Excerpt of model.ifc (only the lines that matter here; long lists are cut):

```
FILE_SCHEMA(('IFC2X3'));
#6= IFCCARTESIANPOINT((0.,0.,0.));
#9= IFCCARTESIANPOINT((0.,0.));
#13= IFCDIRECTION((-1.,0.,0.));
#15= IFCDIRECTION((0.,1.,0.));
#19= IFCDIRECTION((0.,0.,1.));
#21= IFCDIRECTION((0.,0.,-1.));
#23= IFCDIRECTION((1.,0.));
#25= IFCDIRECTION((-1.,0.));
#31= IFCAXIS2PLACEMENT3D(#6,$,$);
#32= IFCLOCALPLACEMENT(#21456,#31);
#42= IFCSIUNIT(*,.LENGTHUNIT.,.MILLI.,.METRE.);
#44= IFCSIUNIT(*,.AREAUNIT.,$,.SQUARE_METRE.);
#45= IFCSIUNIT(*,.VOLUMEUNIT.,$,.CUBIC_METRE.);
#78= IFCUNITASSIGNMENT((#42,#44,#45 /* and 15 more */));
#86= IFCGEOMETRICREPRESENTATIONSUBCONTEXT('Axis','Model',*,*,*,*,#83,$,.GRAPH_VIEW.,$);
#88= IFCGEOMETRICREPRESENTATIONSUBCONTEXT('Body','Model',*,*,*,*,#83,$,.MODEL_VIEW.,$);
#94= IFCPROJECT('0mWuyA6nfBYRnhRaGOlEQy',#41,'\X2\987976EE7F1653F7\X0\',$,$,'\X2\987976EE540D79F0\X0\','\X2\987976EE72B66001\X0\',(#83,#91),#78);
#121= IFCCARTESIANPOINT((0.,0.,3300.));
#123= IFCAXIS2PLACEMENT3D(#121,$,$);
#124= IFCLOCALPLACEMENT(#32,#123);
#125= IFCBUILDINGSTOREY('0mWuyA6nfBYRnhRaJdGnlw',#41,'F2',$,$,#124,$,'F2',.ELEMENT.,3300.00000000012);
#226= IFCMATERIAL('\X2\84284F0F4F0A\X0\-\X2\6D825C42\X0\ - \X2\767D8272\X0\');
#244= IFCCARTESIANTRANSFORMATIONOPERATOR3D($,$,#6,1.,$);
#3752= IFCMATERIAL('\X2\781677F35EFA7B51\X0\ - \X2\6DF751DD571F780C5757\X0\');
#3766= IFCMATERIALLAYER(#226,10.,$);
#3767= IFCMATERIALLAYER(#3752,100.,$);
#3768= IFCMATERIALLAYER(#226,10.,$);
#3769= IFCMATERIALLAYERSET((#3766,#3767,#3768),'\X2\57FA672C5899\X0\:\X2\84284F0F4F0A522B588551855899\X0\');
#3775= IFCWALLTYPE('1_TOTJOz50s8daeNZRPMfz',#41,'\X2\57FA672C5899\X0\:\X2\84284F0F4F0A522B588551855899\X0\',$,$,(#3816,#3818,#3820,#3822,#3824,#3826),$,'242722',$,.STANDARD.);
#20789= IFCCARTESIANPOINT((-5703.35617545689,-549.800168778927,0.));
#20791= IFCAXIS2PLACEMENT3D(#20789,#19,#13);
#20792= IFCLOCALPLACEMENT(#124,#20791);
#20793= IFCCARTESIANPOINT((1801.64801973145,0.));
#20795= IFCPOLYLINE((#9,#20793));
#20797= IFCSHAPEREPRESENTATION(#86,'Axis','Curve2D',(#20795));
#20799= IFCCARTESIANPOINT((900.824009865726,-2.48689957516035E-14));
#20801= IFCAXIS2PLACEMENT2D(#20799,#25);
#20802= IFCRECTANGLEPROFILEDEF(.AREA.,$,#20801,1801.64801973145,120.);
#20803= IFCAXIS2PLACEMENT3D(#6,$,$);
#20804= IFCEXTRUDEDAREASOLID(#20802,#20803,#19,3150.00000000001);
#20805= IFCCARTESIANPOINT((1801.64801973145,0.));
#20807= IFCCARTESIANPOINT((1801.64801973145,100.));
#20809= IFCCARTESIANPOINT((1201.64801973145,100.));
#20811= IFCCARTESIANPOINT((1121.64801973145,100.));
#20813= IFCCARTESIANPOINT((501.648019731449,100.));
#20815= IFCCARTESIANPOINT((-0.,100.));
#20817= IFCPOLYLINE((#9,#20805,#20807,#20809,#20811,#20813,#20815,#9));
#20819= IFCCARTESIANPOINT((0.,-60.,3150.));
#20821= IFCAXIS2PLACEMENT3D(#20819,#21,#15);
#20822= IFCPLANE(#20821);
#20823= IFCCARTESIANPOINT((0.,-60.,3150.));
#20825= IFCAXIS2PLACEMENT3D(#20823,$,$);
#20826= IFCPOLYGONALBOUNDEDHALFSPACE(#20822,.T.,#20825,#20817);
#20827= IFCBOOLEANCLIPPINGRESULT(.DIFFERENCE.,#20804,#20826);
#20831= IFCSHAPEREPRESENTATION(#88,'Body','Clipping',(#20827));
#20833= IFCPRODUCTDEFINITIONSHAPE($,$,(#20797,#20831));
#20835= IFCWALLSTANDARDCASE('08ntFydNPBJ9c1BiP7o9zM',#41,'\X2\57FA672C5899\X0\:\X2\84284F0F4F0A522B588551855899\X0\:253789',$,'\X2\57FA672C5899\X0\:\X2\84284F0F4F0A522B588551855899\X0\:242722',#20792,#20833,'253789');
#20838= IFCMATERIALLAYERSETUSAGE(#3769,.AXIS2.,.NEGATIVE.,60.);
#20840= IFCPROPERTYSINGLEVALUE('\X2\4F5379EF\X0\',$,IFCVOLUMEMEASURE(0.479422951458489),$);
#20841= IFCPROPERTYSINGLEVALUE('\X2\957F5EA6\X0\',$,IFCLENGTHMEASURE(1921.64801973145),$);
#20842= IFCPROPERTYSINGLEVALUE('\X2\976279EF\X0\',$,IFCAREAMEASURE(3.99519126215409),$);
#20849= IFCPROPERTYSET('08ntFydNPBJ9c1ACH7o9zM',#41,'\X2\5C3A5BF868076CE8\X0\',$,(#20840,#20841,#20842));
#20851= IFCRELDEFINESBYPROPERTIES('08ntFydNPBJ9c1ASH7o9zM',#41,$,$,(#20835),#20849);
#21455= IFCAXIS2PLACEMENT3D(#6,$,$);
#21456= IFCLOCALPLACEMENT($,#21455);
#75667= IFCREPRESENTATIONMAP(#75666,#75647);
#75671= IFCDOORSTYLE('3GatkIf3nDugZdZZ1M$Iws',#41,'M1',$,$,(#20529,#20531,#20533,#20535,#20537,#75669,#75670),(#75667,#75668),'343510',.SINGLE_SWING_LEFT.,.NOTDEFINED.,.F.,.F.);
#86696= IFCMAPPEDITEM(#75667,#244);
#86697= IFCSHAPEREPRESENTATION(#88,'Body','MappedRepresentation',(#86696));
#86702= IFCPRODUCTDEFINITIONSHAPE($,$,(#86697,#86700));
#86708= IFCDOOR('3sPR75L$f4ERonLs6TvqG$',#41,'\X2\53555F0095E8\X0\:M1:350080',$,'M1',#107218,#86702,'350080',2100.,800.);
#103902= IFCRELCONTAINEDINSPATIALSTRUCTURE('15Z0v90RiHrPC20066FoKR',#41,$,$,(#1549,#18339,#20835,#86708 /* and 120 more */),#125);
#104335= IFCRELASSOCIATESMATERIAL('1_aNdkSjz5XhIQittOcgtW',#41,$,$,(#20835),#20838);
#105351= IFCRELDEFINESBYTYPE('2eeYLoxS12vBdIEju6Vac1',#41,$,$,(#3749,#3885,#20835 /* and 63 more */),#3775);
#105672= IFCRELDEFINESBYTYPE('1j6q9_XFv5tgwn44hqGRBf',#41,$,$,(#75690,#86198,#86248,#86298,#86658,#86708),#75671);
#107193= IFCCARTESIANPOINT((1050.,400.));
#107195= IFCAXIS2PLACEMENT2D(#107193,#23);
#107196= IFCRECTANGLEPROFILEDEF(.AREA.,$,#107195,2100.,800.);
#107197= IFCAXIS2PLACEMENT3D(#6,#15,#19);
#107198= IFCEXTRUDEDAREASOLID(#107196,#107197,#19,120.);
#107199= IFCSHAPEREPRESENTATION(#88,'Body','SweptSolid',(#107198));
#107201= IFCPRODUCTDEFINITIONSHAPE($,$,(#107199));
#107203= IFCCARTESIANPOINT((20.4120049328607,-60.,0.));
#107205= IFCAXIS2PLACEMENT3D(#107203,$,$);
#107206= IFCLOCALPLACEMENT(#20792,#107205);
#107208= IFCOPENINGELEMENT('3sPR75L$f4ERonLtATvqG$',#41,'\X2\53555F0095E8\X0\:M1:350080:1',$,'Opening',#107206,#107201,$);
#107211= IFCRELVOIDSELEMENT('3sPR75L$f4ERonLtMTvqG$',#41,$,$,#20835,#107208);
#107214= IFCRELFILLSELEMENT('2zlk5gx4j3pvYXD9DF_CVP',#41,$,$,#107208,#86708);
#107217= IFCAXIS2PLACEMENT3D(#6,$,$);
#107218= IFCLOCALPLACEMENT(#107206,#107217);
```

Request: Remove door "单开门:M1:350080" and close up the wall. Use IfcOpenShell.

```python
import ifcopenshell
import ifcopenshell.api.feature
import ifcopenshell.api.pset
import ifcopenshell.api.root
import ifcopenshell.geom
import ifcopenshell.util.element
import ifcopenshell.util.shape
import ifcopenshell.util.unit

model = ifcopenshell.open("model.ifc")
area_scale = ifcopenshell.util.unit.calculate_unit_scale(model, "AREAUNIT")
volume_scale = ifcopenshell.util.unit.calculate_unit_scale(model, "VOLUMEUNIT")
settings = ifcopenshell.geom.settings()


def volume(element):
    """Net volume in cubic metres, openings subtracted."""
    shape = ifcopenshell.geom.create_shape(settings, element)
    return ifcopenshell.util.shape.get_volume(shape.geometry)


door = model.by_guid("3sPR75L$f4ERonLs6TvqG$")
opening = door.FillsVoids[0].RelatingOpeningElement
wall = opening.VoidsElements[0].RelatingBuildingElement
before = volume(wall)

ifcopenshell.api.root.remove_product(model, product=door)
ifcopenshell.api.feature.remove_feature(model, feature=opening)

after = volume(wall)
thickness = 0.12  # wall thickness in metres

# Update the wall's stored quantities.
pset = model.by_id(ifcopenshell.util.element.get_pset(wall, "尺寸标注", should_inherit=False)["id"])
ifcopenshell.api.pset.edit_pset(model, pset=pset, properties={
    "体积": model.create_entity("IfcVolumeMeasure", after / volume_scale),
    "面积": model.create_entity("IfcAreaMeasure", after / thickness / area_scale),
})

print(f"wall volume {before:.3f} -> {after:.3f} m3")

model.write("model-out.ifc")
```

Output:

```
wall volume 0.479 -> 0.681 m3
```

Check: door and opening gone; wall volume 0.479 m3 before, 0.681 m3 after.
